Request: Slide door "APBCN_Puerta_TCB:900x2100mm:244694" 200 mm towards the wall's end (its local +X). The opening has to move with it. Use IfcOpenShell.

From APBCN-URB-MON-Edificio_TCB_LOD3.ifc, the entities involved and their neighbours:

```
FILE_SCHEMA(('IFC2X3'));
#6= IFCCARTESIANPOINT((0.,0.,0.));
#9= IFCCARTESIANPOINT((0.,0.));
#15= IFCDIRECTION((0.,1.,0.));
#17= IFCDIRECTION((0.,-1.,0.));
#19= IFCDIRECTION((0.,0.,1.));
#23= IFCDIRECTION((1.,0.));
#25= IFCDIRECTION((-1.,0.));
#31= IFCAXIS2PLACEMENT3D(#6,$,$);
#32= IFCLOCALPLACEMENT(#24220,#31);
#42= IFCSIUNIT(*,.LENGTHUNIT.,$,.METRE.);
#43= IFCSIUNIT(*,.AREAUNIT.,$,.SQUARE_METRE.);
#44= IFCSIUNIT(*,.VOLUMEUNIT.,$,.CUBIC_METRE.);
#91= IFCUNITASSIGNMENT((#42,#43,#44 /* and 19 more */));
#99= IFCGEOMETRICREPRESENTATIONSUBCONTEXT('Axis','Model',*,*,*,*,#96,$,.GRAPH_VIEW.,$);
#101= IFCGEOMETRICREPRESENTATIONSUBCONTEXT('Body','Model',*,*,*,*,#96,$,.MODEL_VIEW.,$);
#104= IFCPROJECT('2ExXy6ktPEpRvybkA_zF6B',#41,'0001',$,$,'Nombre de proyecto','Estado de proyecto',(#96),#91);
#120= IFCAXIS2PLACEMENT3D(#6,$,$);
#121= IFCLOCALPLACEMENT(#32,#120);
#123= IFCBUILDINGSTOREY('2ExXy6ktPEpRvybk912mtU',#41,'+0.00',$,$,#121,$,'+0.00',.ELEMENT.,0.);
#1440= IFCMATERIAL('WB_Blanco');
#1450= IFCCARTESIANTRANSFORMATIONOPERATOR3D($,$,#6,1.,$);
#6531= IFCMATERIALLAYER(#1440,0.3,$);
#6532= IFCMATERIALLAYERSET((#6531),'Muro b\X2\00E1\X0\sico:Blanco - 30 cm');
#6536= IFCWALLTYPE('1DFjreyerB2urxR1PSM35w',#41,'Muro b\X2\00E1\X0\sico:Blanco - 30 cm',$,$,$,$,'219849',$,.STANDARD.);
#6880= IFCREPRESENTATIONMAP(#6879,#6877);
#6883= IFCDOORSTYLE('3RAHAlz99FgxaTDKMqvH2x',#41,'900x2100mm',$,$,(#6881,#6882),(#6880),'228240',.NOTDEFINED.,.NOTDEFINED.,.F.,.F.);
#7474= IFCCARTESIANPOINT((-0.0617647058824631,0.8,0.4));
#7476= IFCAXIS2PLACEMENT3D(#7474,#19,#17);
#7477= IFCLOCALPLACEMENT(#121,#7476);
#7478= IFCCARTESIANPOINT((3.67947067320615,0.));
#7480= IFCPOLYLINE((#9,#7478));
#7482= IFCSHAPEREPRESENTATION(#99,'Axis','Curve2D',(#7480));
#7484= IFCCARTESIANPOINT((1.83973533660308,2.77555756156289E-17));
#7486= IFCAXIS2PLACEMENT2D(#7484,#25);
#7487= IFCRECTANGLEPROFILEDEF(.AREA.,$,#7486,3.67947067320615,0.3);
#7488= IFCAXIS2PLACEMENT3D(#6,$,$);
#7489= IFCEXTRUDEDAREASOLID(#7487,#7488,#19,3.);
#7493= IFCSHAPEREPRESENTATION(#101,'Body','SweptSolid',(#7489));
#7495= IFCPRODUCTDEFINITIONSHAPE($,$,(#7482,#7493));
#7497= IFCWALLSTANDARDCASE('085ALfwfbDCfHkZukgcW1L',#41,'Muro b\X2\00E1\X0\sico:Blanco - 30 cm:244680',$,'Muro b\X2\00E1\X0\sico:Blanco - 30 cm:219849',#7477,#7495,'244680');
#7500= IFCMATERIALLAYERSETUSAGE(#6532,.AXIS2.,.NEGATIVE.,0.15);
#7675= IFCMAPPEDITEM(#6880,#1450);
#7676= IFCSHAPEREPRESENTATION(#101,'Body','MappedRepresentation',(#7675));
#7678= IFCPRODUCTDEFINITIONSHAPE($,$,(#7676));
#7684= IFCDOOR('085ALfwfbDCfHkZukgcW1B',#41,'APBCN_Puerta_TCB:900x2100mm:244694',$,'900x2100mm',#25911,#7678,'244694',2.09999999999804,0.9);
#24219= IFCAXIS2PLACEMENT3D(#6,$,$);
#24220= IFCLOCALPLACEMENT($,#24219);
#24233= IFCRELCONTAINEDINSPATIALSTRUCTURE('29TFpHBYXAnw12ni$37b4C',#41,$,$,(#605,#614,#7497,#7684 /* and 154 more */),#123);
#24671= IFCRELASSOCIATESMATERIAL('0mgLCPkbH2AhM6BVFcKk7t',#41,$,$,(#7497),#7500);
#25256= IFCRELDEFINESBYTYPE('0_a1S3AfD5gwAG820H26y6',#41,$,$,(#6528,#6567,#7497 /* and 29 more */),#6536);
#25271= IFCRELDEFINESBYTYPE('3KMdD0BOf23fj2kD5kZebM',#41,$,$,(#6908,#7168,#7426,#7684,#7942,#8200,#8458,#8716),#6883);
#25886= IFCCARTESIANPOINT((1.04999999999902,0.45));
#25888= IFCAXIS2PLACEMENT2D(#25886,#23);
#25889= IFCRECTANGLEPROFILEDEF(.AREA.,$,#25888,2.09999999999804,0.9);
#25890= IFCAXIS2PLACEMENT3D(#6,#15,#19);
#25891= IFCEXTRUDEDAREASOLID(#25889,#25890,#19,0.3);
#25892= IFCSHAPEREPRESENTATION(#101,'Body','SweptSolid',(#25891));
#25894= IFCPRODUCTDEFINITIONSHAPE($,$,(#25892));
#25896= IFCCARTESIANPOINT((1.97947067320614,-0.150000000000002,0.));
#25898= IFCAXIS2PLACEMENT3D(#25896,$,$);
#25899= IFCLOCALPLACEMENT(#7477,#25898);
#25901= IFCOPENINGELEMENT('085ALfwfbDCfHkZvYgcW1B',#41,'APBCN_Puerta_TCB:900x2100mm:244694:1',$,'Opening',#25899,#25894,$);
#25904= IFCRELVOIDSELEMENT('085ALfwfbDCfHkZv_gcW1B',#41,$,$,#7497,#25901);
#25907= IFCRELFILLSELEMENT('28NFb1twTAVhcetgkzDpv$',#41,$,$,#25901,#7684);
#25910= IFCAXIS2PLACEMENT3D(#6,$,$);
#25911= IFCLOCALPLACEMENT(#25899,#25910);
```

```python
import ifcopenshell
import ifcopenshell.api.geometry
import ifcopenshell.util.placement
import ifcopenshell.util.unit

model = ifcopenshell.open("APBCN-URB-MON-Edificio_TCB_LOD3.ifc")
unit_scale = ifcopenshell.util.unit.calculate_unit_scale(model)

door = model.by_id(7684)
opening = door.FillsVoids[0].RelatingOpeningElement
wall = opening.VoidsElements[0].RelatingBuildingElement

wall_matrix = ifcopenshell.util.placement.get_local_placement(wall.ObjectPlacement)
shift = wall_matrix[:3, 0] * 0.2 / unit_scale
before = ifcopenshell.util.placement.get_local_placement(door.ObjectPlacement)[:3, 3].copy()

# The door is placed relative to its opening, so it follows when the opening moves.
matrix = ifcopenshell.util.placement.get_local_placement(opening.ObjectPlacement)
matrix[:3, 3] += shift
ifcopenshell.api.geometry.edit_object_placement(
    model, product=opening, matrix=matrix, is_si=False, should_transform_children=True
)

after = ifcopenshell.util.placement.get_local_placement(door.ObjectPlacement)[:3, 3]
print("door moved by", (after - before).round(3) + 0.0)

model.write("APBCN-URB-MON-Edificio_TCB_LOD3_edited.ifc")
```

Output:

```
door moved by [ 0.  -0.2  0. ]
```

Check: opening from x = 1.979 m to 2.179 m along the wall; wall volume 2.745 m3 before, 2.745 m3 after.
